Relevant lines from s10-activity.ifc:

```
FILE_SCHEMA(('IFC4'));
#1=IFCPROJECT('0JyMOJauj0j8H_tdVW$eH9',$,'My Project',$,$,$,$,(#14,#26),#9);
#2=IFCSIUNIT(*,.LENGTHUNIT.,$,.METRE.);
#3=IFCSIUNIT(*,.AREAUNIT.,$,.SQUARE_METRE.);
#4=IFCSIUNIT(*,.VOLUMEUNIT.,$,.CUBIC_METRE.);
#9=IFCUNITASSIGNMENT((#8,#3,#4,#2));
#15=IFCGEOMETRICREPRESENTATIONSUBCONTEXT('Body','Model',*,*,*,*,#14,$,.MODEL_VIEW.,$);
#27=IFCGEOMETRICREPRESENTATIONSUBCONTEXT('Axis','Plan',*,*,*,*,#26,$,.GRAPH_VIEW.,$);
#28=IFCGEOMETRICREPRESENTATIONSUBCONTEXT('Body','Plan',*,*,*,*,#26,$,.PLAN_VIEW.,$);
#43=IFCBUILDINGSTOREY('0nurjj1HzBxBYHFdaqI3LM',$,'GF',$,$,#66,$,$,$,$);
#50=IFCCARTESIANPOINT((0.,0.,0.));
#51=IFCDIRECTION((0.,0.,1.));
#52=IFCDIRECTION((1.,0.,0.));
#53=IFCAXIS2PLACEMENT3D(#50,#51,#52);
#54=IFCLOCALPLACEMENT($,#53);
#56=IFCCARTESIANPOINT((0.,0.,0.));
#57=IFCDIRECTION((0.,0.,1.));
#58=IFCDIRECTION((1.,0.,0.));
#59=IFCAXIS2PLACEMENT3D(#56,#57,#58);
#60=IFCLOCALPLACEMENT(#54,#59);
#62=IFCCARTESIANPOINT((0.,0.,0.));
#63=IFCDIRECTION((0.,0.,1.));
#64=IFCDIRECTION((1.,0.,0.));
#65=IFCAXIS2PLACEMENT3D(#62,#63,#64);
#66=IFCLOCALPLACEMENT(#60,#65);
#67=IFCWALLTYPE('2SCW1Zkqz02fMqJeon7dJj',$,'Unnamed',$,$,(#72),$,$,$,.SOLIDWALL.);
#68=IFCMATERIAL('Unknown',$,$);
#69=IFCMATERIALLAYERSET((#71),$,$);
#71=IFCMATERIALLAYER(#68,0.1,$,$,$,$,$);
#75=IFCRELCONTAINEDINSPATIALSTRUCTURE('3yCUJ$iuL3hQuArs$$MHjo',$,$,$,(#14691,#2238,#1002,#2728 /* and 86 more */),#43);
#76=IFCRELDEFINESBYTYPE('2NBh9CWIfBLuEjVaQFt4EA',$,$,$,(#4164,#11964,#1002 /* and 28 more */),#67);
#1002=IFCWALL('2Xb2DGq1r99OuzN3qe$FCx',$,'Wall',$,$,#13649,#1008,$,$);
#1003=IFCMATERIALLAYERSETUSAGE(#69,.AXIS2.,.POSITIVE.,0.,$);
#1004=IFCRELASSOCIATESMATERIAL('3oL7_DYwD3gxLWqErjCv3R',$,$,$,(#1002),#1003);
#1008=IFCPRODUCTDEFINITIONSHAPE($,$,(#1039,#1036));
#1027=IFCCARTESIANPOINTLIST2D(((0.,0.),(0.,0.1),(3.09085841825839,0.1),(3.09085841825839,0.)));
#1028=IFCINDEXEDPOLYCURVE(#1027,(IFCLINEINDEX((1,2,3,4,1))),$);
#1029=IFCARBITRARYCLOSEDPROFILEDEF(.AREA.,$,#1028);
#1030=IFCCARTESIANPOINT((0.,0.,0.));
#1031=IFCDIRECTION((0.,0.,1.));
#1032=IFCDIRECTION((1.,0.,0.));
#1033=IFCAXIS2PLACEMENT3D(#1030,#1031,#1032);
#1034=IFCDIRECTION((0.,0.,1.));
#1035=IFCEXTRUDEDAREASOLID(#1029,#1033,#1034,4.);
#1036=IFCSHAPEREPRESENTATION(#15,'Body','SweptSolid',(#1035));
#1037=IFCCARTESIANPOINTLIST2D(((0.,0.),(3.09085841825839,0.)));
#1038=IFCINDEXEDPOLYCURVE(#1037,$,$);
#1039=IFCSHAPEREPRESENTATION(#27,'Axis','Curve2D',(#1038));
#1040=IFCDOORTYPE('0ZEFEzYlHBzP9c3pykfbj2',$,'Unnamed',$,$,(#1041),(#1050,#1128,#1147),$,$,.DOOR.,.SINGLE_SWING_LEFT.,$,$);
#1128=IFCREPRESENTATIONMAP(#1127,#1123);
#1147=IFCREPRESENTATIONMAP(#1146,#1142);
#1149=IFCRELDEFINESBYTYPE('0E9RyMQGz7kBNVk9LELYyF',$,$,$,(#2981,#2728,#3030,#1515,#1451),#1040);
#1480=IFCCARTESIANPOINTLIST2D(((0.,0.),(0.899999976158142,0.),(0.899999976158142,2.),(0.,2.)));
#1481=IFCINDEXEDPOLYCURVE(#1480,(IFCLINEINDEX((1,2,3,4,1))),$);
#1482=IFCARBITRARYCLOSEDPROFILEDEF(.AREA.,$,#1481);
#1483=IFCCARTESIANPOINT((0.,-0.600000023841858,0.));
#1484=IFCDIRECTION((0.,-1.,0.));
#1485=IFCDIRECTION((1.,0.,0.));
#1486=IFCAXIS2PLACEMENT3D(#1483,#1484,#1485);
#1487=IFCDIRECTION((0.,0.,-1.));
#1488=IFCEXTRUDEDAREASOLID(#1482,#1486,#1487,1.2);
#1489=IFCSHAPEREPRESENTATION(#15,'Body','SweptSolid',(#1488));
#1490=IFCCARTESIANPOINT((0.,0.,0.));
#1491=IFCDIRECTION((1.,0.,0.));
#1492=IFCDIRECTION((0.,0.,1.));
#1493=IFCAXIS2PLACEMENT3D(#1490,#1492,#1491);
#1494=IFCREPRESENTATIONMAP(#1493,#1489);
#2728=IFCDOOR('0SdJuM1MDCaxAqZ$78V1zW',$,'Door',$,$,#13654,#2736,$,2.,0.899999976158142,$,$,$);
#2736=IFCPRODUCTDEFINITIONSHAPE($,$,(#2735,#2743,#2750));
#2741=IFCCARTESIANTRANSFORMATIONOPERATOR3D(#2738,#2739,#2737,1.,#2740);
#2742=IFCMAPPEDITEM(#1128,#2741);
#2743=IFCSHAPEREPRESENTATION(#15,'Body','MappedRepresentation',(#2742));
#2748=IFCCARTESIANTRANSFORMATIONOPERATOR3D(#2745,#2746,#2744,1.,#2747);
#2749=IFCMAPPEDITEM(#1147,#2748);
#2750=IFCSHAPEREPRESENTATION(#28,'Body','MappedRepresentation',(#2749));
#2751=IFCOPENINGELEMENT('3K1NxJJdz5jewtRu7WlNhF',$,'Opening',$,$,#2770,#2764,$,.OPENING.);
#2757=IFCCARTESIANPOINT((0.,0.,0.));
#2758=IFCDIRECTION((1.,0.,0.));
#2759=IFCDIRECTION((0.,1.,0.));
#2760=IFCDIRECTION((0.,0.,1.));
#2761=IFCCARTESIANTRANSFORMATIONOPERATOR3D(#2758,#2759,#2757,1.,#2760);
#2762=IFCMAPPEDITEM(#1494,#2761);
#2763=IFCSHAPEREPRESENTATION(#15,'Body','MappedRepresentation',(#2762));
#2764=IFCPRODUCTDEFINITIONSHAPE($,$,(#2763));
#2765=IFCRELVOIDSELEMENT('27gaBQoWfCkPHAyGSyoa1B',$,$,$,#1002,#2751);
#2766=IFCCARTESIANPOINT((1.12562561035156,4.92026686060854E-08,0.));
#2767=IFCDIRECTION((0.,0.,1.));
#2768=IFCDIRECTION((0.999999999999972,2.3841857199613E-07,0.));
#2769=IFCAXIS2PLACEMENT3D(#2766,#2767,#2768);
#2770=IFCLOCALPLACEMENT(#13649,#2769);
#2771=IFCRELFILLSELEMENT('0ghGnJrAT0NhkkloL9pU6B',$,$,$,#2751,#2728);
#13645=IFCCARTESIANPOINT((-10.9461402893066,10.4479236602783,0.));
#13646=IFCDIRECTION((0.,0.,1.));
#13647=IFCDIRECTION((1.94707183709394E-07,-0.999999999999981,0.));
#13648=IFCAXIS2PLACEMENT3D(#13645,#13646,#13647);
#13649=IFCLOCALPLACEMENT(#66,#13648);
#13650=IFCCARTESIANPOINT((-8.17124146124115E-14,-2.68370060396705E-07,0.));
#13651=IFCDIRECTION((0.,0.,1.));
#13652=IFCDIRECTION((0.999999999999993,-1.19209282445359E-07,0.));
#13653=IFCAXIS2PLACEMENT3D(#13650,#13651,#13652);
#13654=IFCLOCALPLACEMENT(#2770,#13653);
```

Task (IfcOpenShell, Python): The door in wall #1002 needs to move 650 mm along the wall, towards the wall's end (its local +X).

```python
import ifcopenshell
import ifcopenshell.api.geometry
import ifcopenshell.util.placement
import ifcopenshell.util.unit

model = ifcopenshell.open("s10-activity.ifc")
unit_scale = ifcopenshell.util.unit.calculate_unit_scale(model)

door = model.by_id(2728)
opening = door.FillsVoids[0].RelatingOpeningElement
wall = opening.VoidsElements[0].RelatingBuildingElement

wall_matrix = ifcopenshell.util.placement.get_local_placement(wall.ObjectPlacement)
shift = wall_matrix[:3, 0] * 0.65 / unit_scale
before = ifcopenshell.util.placement.get_local_placement(door.ObjectPlacement)[:3, 3].copy()

# The door is placed relative to its opening, so it follows when the opening moves.
matrix = ifcopenshell.util.placement.get_local_placement(opening.ObjectPlacement)
matrix[:3, 3] += shift
ifcopenshell.api.geometry.edit_object_placement(
    model, product=opening, matrix=matrix, is_si=False, should_transform_children=True
)

after = ifcopenshell.util.placement.get_local_placement(door.ObjectPlacement)[:3, 3]
print("door moved by", (after - before).round(3) + 0.0)

model.write("s10-activity_edited.ifc")
```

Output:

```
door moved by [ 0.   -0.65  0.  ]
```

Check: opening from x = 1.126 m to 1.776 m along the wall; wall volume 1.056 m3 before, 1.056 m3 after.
